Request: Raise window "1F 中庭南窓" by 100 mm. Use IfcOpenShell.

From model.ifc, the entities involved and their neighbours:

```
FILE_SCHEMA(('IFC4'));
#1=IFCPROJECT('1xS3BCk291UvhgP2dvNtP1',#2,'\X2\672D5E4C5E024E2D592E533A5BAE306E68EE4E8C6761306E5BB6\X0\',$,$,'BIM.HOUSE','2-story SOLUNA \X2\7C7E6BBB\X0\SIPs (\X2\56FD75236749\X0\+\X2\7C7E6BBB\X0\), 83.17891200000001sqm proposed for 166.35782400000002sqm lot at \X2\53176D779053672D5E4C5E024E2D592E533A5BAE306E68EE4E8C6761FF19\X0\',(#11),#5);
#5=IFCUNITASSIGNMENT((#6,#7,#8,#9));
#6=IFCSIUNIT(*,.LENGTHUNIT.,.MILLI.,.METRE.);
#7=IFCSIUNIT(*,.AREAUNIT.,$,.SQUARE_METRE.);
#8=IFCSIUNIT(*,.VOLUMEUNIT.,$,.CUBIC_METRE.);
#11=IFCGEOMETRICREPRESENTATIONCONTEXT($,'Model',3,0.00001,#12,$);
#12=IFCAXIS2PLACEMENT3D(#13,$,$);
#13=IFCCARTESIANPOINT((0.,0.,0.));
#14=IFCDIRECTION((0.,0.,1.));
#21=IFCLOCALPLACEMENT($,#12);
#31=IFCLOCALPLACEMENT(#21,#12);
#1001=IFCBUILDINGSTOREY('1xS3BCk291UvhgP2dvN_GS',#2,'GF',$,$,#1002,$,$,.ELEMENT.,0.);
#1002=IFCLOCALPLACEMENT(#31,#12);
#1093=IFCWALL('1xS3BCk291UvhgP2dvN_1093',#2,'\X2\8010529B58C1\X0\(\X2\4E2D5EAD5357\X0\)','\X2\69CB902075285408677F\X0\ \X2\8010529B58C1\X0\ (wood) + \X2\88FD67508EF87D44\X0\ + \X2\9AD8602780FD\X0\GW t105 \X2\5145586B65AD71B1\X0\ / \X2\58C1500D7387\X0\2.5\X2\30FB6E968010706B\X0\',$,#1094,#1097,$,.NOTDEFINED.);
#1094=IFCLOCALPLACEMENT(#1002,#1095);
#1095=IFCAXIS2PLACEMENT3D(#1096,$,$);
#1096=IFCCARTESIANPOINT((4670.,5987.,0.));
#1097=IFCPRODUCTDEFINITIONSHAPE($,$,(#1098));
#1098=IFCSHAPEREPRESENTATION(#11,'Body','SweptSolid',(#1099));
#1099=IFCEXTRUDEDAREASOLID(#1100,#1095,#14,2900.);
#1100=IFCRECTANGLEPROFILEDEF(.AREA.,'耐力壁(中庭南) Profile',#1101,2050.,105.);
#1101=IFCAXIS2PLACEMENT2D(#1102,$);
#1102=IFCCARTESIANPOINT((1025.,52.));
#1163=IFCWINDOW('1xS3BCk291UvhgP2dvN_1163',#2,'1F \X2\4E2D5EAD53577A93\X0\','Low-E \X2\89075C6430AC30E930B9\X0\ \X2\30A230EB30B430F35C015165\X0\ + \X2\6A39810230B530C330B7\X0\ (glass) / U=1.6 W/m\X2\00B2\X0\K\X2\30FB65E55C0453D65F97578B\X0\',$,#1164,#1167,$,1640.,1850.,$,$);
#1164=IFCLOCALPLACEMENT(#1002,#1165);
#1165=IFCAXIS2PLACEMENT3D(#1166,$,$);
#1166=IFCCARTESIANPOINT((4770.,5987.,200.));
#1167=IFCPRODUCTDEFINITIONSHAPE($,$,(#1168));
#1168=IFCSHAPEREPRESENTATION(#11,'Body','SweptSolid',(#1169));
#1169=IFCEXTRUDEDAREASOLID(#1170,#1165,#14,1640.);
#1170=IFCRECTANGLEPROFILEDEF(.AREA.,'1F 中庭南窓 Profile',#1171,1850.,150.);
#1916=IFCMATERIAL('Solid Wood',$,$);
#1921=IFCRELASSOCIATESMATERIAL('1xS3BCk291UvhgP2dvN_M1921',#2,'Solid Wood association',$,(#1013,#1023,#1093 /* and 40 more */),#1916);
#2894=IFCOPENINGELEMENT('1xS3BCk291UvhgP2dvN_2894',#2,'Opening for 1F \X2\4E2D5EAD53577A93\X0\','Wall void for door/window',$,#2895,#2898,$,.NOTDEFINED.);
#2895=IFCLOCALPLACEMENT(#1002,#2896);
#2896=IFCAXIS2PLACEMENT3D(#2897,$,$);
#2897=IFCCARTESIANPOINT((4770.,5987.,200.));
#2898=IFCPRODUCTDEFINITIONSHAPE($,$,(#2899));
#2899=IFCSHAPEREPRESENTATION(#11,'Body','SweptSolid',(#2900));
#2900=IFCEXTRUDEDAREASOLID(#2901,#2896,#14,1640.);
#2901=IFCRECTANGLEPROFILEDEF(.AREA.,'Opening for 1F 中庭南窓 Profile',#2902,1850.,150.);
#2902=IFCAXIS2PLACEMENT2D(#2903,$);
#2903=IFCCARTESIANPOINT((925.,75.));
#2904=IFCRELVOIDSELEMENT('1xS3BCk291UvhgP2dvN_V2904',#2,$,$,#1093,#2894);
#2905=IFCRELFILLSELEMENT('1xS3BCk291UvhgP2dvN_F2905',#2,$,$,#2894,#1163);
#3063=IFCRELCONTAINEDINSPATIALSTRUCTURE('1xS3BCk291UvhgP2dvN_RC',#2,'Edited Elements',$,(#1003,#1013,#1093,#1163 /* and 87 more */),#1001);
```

```python
import numpy as np
import ifcopenshell
import ifcopenshell.api.geometry
import ifcopenshell.util.placement
import ifcopenshell.util.unit

model = ifcopenshell.open("model.ifc")
unit_scale = ifcopenshell.util.unit.calculate_unit_scale(model)

window = model.by_guid("1xS3BCk291UvhgP2dvN_1163")
opening = window.FillsVoids[0].RelatingOpeningElement
dz = 100.0

shift = np.array([0.0, 0.0, dz])
# The window is not placed relative to its opening, so move both.
for product in (opening, window):
    matrix = ifcopenshell.util.placement.get_local_placement(product.ObjectPlacement)
    matrix[:3, 3] += shift
    ifcopenshell.api.geometry.edit_object_placement(model, product=product, matrix=matrix, is_si=False)

print(f"moved by {dz * unit_scale:+.3f} m")

model.write("model-out.ifc")
```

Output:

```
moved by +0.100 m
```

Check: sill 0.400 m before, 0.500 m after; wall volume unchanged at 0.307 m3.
